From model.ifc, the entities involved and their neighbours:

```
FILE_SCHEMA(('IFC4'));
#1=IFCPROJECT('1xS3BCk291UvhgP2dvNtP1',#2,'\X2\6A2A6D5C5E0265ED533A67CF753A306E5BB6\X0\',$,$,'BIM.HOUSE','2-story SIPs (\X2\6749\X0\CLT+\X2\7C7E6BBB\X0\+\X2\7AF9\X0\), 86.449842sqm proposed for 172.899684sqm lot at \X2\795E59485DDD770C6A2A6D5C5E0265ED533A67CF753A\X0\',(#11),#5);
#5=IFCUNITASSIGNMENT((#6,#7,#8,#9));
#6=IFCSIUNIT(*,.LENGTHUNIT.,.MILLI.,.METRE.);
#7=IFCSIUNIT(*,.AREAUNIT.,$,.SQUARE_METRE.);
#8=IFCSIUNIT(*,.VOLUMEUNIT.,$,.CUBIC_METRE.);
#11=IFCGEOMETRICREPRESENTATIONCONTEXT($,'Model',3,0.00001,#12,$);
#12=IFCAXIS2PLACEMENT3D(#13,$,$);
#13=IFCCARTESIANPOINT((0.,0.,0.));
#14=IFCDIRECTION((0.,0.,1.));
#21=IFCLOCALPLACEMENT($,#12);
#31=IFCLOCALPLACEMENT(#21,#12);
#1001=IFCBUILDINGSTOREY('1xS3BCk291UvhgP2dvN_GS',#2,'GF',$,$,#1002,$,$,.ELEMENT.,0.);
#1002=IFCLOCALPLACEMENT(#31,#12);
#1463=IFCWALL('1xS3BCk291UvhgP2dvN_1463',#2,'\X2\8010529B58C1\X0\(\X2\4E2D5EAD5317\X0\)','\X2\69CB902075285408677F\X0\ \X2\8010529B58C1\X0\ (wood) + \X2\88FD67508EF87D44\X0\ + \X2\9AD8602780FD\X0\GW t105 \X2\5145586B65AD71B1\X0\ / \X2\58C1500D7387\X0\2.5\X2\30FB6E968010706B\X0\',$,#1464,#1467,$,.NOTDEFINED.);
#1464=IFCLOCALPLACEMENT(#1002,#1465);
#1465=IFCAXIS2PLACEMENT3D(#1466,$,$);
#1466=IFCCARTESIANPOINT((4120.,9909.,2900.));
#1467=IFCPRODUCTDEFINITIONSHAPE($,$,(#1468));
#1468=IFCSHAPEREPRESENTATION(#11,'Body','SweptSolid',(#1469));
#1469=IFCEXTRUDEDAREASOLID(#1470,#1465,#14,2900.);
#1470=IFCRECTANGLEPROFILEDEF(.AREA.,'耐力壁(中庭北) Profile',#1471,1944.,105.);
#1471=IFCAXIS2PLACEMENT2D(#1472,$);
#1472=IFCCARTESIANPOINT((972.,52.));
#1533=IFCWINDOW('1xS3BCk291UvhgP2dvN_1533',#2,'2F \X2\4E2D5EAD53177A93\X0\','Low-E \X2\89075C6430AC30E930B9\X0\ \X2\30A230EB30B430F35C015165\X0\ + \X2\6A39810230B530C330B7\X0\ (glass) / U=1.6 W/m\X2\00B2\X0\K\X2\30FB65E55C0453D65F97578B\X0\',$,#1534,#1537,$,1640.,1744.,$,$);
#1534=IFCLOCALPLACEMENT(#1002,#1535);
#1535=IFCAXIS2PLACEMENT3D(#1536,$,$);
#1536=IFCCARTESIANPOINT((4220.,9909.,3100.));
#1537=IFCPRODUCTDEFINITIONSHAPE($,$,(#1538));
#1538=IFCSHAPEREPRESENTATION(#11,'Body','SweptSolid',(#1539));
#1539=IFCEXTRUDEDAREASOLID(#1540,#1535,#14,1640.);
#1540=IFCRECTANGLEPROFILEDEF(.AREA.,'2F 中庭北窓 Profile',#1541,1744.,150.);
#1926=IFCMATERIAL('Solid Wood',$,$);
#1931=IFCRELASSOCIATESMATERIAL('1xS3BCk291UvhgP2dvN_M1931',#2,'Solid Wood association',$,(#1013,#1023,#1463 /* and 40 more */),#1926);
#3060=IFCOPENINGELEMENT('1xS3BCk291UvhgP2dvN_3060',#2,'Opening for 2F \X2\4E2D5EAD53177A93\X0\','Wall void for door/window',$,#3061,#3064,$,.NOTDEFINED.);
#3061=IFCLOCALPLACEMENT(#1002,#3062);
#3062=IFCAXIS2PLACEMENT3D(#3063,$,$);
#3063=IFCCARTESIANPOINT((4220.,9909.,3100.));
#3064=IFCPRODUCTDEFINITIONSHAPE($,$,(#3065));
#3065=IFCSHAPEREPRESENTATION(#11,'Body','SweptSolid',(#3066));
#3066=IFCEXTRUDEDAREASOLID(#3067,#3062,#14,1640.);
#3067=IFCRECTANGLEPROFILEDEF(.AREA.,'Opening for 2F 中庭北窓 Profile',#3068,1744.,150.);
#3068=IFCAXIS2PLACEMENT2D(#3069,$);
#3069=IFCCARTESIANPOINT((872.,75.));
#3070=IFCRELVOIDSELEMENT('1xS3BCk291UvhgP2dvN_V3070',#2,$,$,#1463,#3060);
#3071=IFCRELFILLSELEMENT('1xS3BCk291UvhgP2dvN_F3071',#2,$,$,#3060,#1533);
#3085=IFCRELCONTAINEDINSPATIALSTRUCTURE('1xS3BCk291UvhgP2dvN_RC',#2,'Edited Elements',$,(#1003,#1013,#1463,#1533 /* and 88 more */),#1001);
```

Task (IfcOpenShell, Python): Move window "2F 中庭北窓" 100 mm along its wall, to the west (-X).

```python
import ifcopenshell
import ifcopenshell.api.geometry
import ifcopenshell.util.placement
import ifcopenshell.util.unit

model = ifcopenshell.open("model.ifc")
unit_scale = ifcopenshell.util.unit.calculate_unit_scale(model)

window = model.by_guid("1xS3BCk291UvhgP2dvN_1533")
opening = window.FillsVoids[0].RelatingOpeningElement
wall = opening.VoidsElements[0].RelatingBuildingElement

wall_matrix = ifcopenshell.util.placement.get_local_placement(wall.ObjectPlacement)
shift = wall_matrix[:3, 0] * -0.1 / unit_scale
before = ifcopenshell.util.placement.get_local_placement(window.ObjectPlacement)[:3, 3].copy()

# The window is not placed relative to its opening, so move both.
for product in (opening, window):
    matrix = ifcopenshell.util.placement.get_local_placement(product.ObjectPlacement)
    matrix[:3, 3] += shift
    ifcopenshell.api.geometry.edit_object_placement(model, product=product, matrix=matrix, is_si=False)

after = ifcopenshell.util.placement.get_local_placement(window.ObjectPlacement)[:3, 3]
print("window moved by", (after - before).round(3) + 0.0)

model.write("model-out.ifc")
```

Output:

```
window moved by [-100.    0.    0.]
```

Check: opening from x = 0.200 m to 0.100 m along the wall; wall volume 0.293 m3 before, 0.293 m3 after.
